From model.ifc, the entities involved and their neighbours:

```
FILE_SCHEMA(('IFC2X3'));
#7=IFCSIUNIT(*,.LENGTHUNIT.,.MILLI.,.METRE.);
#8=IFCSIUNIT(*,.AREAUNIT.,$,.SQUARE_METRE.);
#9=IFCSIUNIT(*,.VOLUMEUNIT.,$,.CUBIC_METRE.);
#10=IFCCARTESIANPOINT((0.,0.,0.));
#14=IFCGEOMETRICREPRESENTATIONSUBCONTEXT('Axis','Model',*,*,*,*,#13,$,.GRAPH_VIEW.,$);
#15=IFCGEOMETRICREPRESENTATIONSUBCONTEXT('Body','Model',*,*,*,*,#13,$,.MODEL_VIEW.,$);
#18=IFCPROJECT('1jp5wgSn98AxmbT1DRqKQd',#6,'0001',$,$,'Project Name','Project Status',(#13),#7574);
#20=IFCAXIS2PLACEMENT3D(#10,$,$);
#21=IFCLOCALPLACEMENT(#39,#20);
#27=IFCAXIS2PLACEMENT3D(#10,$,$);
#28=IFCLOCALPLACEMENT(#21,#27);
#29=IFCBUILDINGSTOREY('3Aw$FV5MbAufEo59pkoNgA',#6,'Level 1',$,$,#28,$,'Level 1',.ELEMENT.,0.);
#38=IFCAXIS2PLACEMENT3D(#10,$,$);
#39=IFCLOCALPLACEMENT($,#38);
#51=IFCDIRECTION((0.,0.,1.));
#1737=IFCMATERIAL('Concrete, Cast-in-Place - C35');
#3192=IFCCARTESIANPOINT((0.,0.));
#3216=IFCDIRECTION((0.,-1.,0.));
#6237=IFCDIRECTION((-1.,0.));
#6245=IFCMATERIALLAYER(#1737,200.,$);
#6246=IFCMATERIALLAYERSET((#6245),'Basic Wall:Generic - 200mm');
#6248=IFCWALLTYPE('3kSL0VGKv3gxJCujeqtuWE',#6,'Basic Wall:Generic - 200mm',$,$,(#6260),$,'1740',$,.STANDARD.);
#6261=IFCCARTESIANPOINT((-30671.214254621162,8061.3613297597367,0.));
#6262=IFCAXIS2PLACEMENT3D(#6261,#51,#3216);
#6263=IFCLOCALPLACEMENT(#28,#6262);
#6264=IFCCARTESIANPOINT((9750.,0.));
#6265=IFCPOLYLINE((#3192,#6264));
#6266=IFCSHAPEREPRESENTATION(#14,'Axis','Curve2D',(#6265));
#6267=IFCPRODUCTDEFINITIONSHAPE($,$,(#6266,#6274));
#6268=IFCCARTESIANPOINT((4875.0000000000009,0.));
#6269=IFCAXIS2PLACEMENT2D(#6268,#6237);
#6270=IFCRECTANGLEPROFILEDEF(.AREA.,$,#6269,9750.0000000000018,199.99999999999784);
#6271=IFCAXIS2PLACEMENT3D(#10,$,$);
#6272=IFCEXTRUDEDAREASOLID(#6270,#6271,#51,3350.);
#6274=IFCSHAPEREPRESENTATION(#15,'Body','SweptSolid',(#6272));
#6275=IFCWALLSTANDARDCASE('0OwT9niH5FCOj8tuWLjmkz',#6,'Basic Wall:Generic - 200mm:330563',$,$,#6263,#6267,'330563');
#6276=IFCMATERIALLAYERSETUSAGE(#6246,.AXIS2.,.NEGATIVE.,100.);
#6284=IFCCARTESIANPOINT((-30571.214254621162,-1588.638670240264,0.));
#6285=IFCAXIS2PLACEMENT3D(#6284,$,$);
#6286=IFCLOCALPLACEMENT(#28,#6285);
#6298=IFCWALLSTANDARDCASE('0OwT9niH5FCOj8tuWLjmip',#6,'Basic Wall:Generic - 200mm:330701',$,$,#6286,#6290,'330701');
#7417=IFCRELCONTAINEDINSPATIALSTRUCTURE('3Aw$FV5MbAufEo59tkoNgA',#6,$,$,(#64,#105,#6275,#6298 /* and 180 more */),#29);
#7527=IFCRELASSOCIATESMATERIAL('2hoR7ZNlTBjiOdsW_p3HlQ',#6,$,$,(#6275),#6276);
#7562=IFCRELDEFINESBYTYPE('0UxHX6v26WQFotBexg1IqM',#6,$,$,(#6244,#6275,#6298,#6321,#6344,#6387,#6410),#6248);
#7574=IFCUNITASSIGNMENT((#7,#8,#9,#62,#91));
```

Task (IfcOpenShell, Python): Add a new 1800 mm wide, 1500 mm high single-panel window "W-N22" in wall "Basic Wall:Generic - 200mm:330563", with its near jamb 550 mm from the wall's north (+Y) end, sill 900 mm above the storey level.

```python
import numpy as np
import ifcopenshell
import ifcopenshell.api.feature
import ifcopenshell.api.geometry
import ifcopenshell.api.root
import ifcopenshell.api.spatial
import ifcopenshell.api.type
import ifcopenshell.geom
import ifcopenshell.util.element
import ifcopenshell.util.placement
import ifcopenshell.util.representation
import ifcopenshell.util.shape
import ifcopenshell.util.unit

model = ifcopenshell.open("model.ifc")
unit_scale = ifcopenshell.util.unit.calculate_unit_scale(model)
settings = ifcopenshell.geom.settings()


def volume(element):
    """Net volume in cubic metres, openings subtracted."""
    shape = ifcopenshell.geom.create_shape(settings, element)
    return ifcopenshell.util.shape.get_volume(shape.geometry)


wall = model.by_id(6275)
storey = ifcopenshell.util.element.get_container(wall, ifc_class="IfcBuildingStorey")
context = ifcopenshell.util.representation.get_context(model, "Model", "Body", "MODEL_VIEW")
before = volume(wall)

width, height, from_end, sill = 1.8, 1.5, 0.55, 0.9  # metres

# The wall runs along its own X axis, and the end named is its -X end.
wall_shape = ifcopenshell.geom.create_shape(settings, wall)
x, y, z = ifcopenshell.util.shape.get_vertices(wall_shape.geometry).T
start = x.min() + from_end
face, thickness = float(y.min()), float(y.max() - y.min())
wall_matrix = ifcopenshell.util.placement.get_local_placement(wall.ObjectPlacement)
level = ifcopenshell.util.placement.get_local_placement(storey.ObjectPlacement)[2, 3]


def in_wall(x, y):
    """Placement at x, y metres in the wall's axes, at sill height."""
    matrix = wall_matrix.copy()
    matrix[:, 3] = wall_matrix @ np.array([x / unit_scale, y / unit_scale, 0.0, 1.0])
    matrix[2, 3] = level + sill / unit_scale
    return matrix


# Opening: a box that overshoots both wall faces by 50 mm.
opening = ifcopenshell.api.root.create_entity(model, ifc_class="IfcOpeningElement")
box = ifcopenshell.api.geometry.add_wall_representation(
    model, context=context, length=width, height=height, thickness=thickness + 0.1
)
ifcopenshell.api.geometry.assign_representation(model, product=opening, representation=box)
ifcopenshell.api.geometry.edit_object_placement(model, product=opening, matrix=in_wall(start, face - 0.05), is_si=False)
ifcopenshell.api.feature.add_feature(model, feature=opening, element=wall)

window = ifcopenshell.api.root.create_entity(model, ifc_class="IfcWindow", name="W-N22")
window.OverallWidth, window.OverallHeight = width / unit_scale, height / unit_scale
body = ifcopenshell.api.geometry.add_window_representation(
    model,
    context=context,
    overall_width=window.OverallWidth,
    overall_height=window.OverallHeight,
    partition_type="SINGLE_PANEL",
)
ifcopenshell.api.geometry.assign_representation(model, product=window, representation=body)
ifcopenshell.api.spatial.assign_container(model, products=[window], relating_structure=storey)
fills = ifcopenshell.api.feature.add_filling(model, opening=opening, element=window)
fills.OwnerHistory = window.OwnerHistory  # required in IFC2X3

# IFC2X3 keeps the operation on the window style.
style = ifcopenshell.api.root.create_entity(model, ifc_class="IfcWindowStyle", name="W-N22")
style.OperationType, style.ConstructionType = "SINGLE_PANEL", "NOTDEFINED"
style.ParameterTakesPrecedence = style.Sizeable = False
ifcopenshell.api.type.assign_type(model, related_objects=[window], relating_type=style)

# Centre the window in the wall's thickness.
ifcopenshell.api.geometry.edit_object_placement(model, product=window, matrix=in_wall(start, face), is_si=False)
window_shape = ifcopenshell.geom.create_shape(settings, window)
depth = ifcopenshell.util.shape.get_vertices(window_shape.geometry)[:, 1]
offset = face + thickness / 2 - (depth.min() + depth.max()) / 2
ifcopenshell.api.geometry.edit_object_placement(model, product=window, matrix=in_wall(start, offset), is_si=False)

after = volume(wall)

print(f"wall volume {before:.3f} -> {after:.3f} m3")

model.write("model_edited.ifc")
```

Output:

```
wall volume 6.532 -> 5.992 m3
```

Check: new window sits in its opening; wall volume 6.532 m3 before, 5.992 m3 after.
